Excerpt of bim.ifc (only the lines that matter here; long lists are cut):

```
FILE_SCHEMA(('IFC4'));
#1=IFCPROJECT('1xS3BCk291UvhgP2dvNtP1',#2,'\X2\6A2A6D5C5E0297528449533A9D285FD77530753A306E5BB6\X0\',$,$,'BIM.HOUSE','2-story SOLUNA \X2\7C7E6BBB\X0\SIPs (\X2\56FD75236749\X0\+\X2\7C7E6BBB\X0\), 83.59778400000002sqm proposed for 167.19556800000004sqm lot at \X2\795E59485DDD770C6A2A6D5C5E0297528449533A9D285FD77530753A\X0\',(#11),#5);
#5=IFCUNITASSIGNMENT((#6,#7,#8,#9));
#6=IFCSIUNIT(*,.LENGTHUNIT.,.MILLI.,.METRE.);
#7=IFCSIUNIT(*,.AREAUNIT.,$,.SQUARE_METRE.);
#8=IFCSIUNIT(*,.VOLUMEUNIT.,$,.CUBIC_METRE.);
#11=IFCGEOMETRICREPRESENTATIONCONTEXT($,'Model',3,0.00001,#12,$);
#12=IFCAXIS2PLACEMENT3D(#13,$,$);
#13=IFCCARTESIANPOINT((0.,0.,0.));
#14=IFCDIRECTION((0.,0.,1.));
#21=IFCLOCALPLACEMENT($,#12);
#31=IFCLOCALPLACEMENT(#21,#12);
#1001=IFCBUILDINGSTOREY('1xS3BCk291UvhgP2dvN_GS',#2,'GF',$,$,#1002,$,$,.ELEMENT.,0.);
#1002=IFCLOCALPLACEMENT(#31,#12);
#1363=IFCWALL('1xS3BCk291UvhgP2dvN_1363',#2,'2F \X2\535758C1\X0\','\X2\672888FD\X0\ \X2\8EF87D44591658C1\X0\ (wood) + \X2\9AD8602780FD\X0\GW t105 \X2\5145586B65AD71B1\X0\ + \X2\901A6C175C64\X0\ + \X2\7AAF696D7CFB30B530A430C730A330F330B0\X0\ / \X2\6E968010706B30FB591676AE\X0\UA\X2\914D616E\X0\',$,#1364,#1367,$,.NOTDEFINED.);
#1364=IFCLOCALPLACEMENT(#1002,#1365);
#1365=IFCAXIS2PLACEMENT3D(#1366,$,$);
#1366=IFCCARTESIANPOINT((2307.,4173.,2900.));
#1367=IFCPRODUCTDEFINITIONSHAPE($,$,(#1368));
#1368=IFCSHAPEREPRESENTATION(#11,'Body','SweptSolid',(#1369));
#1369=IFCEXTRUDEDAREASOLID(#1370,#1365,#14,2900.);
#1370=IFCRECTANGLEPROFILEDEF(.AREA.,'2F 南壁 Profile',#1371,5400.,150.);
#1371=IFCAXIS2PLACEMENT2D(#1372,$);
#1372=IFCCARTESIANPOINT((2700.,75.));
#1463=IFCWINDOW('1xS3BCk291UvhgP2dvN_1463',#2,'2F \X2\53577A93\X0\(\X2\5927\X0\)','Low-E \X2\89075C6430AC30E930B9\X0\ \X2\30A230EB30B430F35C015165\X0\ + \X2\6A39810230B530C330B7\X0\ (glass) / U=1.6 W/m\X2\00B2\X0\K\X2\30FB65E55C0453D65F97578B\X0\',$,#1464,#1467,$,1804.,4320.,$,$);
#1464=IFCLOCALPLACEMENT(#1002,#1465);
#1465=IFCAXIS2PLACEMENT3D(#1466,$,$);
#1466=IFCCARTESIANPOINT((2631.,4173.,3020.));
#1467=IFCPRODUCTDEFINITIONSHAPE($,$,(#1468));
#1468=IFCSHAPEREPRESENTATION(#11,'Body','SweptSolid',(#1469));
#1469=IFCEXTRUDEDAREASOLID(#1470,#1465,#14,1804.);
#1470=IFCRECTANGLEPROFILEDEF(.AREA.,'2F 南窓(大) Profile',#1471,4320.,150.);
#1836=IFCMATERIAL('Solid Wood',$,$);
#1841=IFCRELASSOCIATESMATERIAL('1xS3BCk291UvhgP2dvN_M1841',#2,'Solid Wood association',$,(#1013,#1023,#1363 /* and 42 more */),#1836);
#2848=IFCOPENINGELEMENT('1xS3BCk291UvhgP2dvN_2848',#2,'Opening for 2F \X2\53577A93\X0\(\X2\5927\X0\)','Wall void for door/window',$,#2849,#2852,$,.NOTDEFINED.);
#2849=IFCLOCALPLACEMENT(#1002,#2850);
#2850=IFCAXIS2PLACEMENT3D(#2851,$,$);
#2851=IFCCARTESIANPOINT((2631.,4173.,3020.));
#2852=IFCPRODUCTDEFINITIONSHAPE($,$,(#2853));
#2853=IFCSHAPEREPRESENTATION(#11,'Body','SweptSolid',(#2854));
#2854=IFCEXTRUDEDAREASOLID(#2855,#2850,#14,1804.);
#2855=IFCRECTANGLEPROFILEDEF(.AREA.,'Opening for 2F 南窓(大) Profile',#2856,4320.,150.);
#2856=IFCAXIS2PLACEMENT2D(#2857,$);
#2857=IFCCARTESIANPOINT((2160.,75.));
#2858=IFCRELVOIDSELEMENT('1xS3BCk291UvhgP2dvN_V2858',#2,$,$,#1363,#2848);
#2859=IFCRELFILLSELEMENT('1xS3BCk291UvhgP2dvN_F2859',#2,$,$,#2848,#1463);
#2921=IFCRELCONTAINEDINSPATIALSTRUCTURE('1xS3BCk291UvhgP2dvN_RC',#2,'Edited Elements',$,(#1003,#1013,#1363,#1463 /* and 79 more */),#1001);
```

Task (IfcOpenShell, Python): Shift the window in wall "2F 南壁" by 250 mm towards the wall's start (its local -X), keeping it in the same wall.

```python
import ifcopenshell
import ifcopenshell.api.geometry
import ifcopenshell.util.placement

model = ifcopenshell.open("bim.ifc")

window = model.by_guid("1xS3BCk291UvhgP2dvN_1463")
opening = window.FillsVoids[0].RelatingOpeningElement
wall = opening.VoidsElements[0].RelatingBuildingElement

wall_matrix = ifcopenshell.util.placement.get_local_placement(wall.ObjectPlacement)
shift = wall_matrix[:3, 0] * -250.0
before = ifcopenshell.util.placement.get_local_placement(window.ObjectPlacement)[:3, 3].copy()

# The window is not placed relative to its opening, so move both.
for product in (opening, window):
    matrix = ifcopenshell.util.placement.get_local_placement(product.ObjectPlacement)
    matrix[:3, 3] += shift
    ifcopenshell.api.geometry.edit_object_placement(model, product=product, matrix=matrix, is_si=False)

after = ifcopenshell.util.placement.get_local_placement(window.ObjectPlacement)[:3, 3]
print("window moved by", (after - before).round(3) + 0.0)

model.write("bim_updated.ifc")
```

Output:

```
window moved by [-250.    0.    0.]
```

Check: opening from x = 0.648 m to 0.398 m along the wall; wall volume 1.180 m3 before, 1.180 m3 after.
